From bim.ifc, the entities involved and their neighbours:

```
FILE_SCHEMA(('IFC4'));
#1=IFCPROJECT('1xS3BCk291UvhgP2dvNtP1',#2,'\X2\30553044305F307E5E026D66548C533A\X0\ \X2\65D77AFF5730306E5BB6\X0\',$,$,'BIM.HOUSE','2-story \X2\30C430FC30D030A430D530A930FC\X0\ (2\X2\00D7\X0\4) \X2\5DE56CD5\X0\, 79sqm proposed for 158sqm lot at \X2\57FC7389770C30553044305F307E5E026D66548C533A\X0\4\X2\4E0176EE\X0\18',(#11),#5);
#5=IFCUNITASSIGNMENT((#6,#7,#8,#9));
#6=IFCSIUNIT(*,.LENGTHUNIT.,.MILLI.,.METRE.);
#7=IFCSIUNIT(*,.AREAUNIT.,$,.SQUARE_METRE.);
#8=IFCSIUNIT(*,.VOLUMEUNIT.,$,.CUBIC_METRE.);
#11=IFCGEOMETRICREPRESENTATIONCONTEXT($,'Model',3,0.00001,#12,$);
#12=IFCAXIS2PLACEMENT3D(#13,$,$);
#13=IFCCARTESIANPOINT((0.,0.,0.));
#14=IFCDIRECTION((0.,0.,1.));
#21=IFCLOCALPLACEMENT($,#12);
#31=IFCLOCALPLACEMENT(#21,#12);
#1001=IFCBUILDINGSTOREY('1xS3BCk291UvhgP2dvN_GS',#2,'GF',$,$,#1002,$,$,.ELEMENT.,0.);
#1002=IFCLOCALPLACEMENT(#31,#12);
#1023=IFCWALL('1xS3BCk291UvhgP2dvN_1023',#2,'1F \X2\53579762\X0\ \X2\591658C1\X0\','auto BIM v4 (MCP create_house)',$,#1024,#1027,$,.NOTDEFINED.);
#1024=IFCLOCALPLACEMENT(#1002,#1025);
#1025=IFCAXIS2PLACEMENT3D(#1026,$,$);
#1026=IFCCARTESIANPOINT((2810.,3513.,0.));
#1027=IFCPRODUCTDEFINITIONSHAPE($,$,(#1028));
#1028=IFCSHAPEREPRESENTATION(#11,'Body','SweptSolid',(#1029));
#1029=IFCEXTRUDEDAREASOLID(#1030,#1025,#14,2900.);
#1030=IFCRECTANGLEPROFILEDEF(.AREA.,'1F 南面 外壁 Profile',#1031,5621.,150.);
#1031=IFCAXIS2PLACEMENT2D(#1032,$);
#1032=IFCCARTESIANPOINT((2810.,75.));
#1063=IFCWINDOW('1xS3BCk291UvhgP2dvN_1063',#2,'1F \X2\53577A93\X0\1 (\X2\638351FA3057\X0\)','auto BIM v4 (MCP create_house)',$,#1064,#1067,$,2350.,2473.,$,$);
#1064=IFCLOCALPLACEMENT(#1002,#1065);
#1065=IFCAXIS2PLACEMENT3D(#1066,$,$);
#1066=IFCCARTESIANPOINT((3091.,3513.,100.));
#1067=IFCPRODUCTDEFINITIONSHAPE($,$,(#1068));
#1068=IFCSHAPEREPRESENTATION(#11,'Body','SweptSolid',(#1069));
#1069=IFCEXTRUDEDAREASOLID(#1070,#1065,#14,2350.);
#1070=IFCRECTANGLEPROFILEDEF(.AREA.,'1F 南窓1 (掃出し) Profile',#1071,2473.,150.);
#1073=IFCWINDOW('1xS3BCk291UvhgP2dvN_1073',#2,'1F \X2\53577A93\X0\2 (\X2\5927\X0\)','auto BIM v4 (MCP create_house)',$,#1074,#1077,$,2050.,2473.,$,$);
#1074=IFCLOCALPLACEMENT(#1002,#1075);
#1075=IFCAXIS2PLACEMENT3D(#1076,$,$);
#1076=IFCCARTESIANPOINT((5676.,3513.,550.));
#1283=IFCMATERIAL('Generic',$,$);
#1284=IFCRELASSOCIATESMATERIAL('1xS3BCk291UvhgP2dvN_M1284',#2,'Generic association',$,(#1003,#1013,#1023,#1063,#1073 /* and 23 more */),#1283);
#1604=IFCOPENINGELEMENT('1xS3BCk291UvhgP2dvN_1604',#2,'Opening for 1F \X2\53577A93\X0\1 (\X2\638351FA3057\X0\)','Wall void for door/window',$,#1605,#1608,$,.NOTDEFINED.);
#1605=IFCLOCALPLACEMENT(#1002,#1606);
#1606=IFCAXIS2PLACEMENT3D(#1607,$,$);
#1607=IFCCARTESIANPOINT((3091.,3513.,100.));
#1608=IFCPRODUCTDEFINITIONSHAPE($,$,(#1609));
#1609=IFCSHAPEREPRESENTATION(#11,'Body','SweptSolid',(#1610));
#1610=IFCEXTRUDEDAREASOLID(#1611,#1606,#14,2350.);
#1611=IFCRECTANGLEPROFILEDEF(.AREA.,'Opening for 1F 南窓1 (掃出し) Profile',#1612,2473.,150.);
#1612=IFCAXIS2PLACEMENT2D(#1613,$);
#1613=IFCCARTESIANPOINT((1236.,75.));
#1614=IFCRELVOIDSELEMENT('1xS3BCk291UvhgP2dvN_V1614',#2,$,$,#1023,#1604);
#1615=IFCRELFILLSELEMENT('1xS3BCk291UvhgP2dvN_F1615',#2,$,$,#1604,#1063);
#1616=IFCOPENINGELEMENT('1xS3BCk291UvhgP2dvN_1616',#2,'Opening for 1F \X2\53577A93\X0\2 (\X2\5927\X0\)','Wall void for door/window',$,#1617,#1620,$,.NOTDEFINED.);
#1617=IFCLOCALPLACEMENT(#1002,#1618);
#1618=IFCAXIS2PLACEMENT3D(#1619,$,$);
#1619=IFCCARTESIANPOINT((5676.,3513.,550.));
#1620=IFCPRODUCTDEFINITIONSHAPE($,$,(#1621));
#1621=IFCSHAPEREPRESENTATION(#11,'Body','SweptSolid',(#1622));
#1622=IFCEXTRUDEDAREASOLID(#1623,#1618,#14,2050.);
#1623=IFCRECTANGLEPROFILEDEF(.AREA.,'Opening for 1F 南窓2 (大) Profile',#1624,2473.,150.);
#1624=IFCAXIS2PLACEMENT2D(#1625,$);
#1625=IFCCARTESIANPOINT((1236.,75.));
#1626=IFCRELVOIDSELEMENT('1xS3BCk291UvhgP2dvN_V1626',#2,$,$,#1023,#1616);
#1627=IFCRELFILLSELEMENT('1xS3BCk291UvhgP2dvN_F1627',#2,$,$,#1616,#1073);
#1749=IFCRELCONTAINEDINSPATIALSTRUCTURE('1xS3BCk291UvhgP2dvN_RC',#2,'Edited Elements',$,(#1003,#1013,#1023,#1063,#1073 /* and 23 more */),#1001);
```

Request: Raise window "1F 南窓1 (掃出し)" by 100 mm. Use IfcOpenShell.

```python
import numpy as np
import ifcopenshell
import ifcopenshell.api.geometry
import ifcopenshell.util.placement
import ifcopenshell.util.unit

model = ifcopenshell.open("bim.ifc")
unit_scale = ifcopenshell.util.unit.calculate_unit_scale(model)

window = model.by_id(1063)
opening = window.FillsVoids[0].RelatingOpeningElement
dz = 100.0

shift = np.array([0.0, 0.0, dz])
# The window is not placed relative to its opening, so move both.
for product in (opening, window):
    matrix = ifcopenshell.util.placement.get_local_placement(product.ObjectPlacement)
    matrix[:3, 3] += shift
    ifcopenshell.api.geometry.edit_object_placement(model, product=product, matrix=matrix, is_si=False)

print(f"moved by {dz * unit_scale:+.3f} m")

model.write("bim-out.ifc")
```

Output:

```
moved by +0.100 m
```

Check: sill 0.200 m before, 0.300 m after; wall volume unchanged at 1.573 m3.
